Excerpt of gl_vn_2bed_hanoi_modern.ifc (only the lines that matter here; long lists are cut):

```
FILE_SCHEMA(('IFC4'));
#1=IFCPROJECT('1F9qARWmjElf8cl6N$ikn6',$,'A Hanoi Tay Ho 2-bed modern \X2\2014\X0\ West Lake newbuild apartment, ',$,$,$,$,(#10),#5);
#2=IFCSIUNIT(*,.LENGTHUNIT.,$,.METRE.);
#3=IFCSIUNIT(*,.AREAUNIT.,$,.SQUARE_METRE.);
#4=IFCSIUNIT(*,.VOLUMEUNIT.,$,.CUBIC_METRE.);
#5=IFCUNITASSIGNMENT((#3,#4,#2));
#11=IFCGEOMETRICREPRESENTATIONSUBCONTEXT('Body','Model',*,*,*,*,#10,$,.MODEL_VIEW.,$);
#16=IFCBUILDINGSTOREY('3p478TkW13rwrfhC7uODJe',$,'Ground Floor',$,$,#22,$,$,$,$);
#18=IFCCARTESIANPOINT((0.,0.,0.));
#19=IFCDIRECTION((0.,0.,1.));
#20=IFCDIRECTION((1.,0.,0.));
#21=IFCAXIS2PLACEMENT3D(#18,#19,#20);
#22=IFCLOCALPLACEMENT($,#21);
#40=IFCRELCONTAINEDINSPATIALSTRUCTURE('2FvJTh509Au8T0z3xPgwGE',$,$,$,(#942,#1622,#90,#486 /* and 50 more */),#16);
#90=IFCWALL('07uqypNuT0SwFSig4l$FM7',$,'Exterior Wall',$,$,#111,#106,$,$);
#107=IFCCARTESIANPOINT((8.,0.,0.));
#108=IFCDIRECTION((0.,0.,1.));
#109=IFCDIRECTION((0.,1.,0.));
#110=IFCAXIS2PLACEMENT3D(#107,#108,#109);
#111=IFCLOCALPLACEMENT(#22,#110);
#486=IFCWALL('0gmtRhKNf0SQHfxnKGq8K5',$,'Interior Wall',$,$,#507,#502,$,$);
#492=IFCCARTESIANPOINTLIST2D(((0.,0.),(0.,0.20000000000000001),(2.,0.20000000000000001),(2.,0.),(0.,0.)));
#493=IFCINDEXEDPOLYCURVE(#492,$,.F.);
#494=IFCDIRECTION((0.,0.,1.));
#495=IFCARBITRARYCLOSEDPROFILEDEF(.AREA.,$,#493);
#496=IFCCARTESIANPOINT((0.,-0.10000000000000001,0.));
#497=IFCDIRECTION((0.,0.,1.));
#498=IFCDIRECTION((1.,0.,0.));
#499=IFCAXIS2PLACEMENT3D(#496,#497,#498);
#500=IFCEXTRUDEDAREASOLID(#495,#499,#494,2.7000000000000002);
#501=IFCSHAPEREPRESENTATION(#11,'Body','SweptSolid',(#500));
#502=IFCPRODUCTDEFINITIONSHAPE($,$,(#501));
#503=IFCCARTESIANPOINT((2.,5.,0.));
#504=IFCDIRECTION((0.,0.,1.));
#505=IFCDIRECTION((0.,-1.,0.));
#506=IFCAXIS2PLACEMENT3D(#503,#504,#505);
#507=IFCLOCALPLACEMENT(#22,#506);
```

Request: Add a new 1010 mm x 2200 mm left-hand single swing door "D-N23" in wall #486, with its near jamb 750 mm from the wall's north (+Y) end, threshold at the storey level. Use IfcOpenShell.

```python
import numpy as np
import ifcopenshell
import ifcopenshell.api.feature
import ifcopenshell.api.geometry
import ifcopenshell.api.root
import ifcopenshell.api.spatial
import ifcopenshell.geom
import ifcopenshell.util.element
import ifcopenshell.util.placement
import ifcopenshell.util.representation
import ifcopenshell.util.shape
import ifcopenshell.util.unit

model = ifcopenshell.open("gl_vn_2bed_hanoi_modern.ifc")
unit_scale = ifcopenshell.util.unit.calculate_unit_scale(model)
settings = ifcopenshell.geom.settings()


def volume(element):
    """Net volume in cubic metres, openings subtracted."""
    shape = ifcopenshell.geom.create_shape(settings, element)
    return ifcopenshell.util.shape.get_volume(shape.geometry)


wall = model.by_guid("0gmtRhKNf0SQHfxnKGq8K5")
storey = ifcopenshell.util.element.get_container(wall, ifc_class="IfcBuildingStorey")
context = ifcopenshell.util.representation.get_context(model, "Model", "Body", "MODEL_VIEW")
before = volume(wall)

width, height, from_end, sill = 1.01, 2.2, 0.75, 0.0  # metres

# The wall runs along its own X axis, and the end named is its -X end.
wall_shape = ifcopenshell.geom.create_shape(settings, wall)
x, y, z = ifcopenshell.util.shape.get_vertices(wall_shape.geometry).T
start = x.min() + from_end
face, thickness = float(y.min()), float(y.max() - y.min())
wall_matrix = ifcopenshell.util.placement.get_local_placement(wall.ObjectPlacement)
level = ifcopenshell.util.placement.get_local_placement(storey.ObjectPlacement)[2, 3]


def in_wall(x, y):
    """Placement at x, y metres in the wall's axes, at sill height."""
    matrix = wall_matrix.copy()
    matrix[:, 3] = wall_matrix @ np.array([x / unit_scale, y / unit_scale, 0.0, 1.0])
    matrix[2, 3] = level + sill / unit_scale
    return matrix


# Opening: a box that overshoots both wall faces by 50 mm.
opening = ifcopenshell.api.root.create_entity(model, ifc_class="IfcOpeningElement", predefined_type="OPENING")
box = ifcopenshell.api.geometry.add_wall_representation(
    model, context=context, length=width, height=height, thickness=thickness + 0.1
)
ifcopenshell.api.geometry.assign_representation(model, product=opening, representation=box)
ifcopenshell.api.geometry.edit_object_placement(model, product=opening, matrix=in_wall(start, face - 0.05), is_si=False)
ifcopenshell.api.feature.add_feature(model, feature=opening, element=wall)

door = ifcopenshell.api.root.create_entity(model, ifc_class="IfcDoor", name="D-N23", predefined_type="DOOR")
door.OverallWidth, door.OverallHeight = width / unit_scale, height / unit_scale
door.OperationType = "SINGLE_SWING_LEFT"
body = ifcopenshell.api.geometry.add_door_representation(
    model,
    context=context,
    overall_width=door.OverallWidth,
    overall_height=door.OverallHeight,
    operation_type="SINGLE_SWING_LEFT",
    lining_properties={"LiningDepth": thickness / unit_scale, "ThresholdDepth": thickness / unit_scale},
)
ifcopenshell.api.geometry.assign_representation(model, product=door, representation=body)
ifcopenshell.api.spatial.assign_container(model, products=[door], relating_structure=storey)
ifcopenshell.api.feature.add_filling(model, opening=opening, element=door)

# The lining spans the wall, so the door starts at the wall face.
ifcopenshell.api.geometry.edit_object_placement(model, product=door, matrix=in_wall(start, face), is_si=False)

after = volume(wall)

print(f"wall volume {before:.3f} -> {after:.3f} m3")

model.write("gl_vn_2bed_hanoi_modern_updated.ifc")
```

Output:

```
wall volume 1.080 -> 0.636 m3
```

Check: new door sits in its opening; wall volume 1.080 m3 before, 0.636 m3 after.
